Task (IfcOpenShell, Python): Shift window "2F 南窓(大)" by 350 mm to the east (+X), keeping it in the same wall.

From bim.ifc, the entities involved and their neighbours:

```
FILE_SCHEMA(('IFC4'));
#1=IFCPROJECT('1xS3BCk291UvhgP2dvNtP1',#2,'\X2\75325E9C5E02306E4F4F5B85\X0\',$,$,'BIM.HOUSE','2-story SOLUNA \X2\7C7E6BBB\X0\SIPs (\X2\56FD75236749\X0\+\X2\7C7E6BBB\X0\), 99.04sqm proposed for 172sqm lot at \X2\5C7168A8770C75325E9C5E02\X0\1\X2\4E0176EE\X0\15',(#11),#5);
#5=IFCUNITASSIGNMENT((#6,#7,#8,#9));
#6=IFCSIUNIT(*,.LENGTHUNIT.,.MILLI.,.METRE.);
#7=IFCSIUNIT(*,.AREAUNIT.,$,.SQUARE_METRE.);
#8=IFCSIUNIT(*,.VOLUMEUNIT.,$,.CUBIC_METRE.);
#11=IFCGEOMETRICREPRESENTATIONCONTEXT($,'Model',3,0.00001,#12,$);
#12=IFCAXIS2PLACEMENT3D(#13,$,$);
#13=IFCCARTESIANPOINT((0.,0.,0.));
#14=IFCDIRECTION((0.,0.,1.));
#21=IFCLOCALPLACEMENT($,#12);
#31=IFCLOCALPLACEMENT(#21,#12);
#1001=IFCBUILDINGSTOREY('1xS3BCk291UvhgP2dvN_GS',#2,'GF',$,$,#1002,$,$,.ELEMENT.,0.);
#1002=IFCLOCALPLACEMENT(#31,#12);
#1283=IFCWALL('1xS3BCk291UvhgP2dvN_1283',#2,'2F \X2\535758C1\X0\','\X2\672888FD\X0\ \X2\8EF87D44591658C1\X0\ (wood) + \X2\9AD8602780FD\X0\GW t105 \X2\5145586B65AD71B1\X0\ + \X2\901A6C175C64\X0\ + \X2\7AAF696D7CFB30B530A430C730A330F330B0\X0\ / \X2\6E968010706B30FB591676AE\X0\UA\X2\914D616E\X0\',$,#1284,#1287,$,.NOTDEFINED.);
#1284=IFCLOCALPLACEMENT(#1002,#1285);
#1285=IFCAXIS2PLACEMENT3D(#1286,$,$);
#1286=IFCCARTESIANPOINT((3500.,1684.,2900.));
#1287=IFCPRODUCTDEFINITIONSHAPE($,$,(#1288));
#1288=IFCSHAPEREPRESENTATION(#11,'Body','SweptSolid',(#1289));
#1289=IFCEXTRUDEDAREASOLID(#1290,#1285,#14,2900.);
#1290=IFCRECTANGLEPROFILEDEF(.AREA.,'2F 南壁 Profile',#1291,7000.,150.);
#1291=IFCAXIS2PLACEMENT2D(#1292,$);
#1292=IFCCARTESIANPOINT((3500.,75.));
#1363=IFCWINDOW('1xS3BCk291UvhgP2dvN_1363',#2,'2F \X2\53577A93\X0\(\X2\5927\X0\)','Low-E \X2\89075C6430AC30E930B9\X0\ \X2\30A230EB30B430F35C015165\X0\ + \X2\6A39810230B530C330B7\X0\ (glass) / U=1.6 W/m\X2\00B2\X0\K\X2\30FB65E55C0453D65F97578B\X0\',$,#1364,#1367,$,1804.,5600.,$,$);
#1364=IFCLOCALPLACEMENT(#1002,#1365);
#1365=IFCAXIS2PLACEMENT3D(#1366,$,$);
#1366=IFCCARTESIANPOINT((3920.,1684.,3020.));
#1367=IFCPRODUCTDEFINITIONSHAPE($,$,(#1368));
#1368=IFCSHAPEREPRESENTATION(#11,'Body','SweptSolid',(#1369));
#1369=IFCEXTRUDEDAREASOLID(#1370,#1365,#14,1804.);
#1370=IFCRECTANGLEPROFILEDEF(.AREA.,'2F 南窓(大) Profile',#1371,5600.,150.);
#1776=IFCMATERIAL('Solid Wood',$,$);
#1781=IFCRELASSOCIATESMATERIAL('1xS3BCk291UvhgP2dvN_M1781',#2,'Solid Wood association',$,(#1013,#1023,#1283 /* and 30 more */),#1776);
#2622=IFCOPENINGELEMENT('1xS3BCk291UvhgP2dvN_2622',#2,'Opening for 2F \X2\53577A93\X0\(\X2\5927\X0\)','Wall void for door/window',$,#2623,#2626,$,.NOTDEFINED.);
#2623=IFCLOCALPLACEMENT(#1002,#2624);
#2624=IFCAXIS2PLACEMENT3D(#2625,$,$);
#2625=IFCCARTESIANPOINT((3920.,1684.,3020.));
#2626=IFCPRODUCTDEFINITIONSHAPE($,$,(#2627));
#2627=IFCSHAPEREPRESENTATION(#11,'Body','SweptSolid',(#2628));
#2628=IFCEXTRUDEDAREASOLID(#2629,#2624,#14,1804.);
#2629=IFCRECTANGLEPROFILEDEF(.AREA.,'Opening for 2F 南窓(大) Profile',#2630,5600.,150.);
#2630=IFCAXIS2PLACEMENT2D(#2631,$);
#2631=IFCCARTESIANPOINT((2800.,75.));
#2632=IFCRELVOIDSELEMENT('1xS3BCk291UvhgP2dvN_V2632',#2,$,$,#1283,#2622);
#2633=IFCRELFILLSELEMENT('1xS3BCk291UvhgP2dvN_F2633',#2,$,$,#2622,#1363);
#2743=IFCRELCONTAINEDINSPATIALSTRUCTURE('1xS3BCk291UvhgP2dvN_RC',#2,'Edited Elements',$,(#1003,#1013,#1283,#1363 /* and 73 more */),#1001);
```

```python
import ifcopenshell
import ifcopenshell.api.geometry
import ifcopenshell.util.placement
import ifcopenshell.util.unit

model = ifcopenshell.open("bim.ifc")
unit_scale = ifcopenshell.util.unit.calculate_unit_scale(model)

window = model.by_guid("1xS3BCk291UvhgP2dvN_1363")
opening = window.FillsVoids[0].RelatingOpeningElement
wall = opening.VoidsElements[0].RelatingBuildingElement

wall_matrix = ifcopenshell.util.placement.get_local_placement(wall.ObjectPlacement)
shift = wall_matrix[:3, 0] * 0.35 / unit_scale
before = ifcopenshell.util.placement.get_local_placement(window.ObjectPlacement)[:3, 3].copy()

# The window is not placed relative to its opening, so move both.
for product in (opening, window):
    matrix = ifcopenshell.util.placement.get_local_placement(product.ObjectPlacement)
    matrix[:3, 3] += shift
    ifcopenshell.api.geometry.edit_object_placement(model, product=product, matrix=matrix, is_si=False)

after = ifcopenshell.util.placement.get_local_placement(window.ObjectPlacement)[:3, 3]
print("window moved by", (after - before).round(3) + 0.0)

model.write("bim_edited.ifc")
```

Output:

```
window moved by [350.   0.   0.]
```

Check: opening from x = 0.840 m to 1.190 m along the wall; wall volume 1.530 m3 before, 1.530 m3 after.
